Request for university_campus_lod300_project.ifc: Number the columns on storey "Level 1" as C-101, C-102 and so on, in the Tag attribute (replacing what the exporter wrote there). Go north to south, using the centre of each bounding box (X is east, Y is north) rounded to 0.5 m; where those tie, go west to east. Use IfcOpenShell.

First a look at what the model holds.

```python
import ifcopenshell
import ifcopenshell.util.element
import ifcopenshell.util.placement

model = ifcopenshell.open("university_campus_lod300_project.ifc")
print(model.schema)
storey = next(s for s in model.by_type("IfcBuildingStorey") if s.Name == "Level 1")
columns = [e for e in ifcopenshell.util.element.get_decomposition(storey) if e.is_a("IfcColumn")]
for e in sorted(columns, key=lambda e: e.id()):
    origin = ifcopenshell.util.placement.get_local_placement(e.ObjectPlacement)[:3, 3]
    print(e.id(), e.Tag, e.Name, origin.round(2) + 0.0, sep=" | ")
```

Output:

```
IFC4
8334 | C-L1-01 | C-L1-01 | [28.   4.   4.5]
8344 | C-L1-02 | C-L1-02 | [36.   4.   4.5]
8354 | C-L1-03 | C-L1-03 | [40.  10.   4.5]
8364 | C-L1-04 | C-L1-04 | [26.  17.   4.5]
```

```python
import ifcopenshell
import ifcopenshell.geom
import ifcopenshell.util.element
import ifcopenshell.util.shape

model = ifcopenshell.open("university_campus_lod300_project.ifc")
settings = ifcopenshell.geom.settings()
settings.set("use-world-coords", True)


def centre(element):
    shape = ifcopenshell.geom.create_shape(settings, element)
    return ifcopenshell.util.shape.get_bbox_centroid(shape.geometry)


storey = next(s for s in model.by_type("IfcBuildingStorey") if s.Name == "Level 1")
columns = [e for e in ifcopenshell.util.element.get_decomposition(storey) if e.is_a("IfcColumn")]

# Insertion points can sit at a corner or the storey origin, so sort by the geometry (in metres).
centres = {e: centre(e) for e in columns}
columns.sort(key=lambda e: (-round(centres[e][1] / 0.5), centres[e][0]))

for i, e in enumerate(columns, start=1):
    number = f"C-1{i:02d}"
    e.Tag = number
    print(e.id(), number)

model.write("university_campus_lod300_project_v2.ifc")
```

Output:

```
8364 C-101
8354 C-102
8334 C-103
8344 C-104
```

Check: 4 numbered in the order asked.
